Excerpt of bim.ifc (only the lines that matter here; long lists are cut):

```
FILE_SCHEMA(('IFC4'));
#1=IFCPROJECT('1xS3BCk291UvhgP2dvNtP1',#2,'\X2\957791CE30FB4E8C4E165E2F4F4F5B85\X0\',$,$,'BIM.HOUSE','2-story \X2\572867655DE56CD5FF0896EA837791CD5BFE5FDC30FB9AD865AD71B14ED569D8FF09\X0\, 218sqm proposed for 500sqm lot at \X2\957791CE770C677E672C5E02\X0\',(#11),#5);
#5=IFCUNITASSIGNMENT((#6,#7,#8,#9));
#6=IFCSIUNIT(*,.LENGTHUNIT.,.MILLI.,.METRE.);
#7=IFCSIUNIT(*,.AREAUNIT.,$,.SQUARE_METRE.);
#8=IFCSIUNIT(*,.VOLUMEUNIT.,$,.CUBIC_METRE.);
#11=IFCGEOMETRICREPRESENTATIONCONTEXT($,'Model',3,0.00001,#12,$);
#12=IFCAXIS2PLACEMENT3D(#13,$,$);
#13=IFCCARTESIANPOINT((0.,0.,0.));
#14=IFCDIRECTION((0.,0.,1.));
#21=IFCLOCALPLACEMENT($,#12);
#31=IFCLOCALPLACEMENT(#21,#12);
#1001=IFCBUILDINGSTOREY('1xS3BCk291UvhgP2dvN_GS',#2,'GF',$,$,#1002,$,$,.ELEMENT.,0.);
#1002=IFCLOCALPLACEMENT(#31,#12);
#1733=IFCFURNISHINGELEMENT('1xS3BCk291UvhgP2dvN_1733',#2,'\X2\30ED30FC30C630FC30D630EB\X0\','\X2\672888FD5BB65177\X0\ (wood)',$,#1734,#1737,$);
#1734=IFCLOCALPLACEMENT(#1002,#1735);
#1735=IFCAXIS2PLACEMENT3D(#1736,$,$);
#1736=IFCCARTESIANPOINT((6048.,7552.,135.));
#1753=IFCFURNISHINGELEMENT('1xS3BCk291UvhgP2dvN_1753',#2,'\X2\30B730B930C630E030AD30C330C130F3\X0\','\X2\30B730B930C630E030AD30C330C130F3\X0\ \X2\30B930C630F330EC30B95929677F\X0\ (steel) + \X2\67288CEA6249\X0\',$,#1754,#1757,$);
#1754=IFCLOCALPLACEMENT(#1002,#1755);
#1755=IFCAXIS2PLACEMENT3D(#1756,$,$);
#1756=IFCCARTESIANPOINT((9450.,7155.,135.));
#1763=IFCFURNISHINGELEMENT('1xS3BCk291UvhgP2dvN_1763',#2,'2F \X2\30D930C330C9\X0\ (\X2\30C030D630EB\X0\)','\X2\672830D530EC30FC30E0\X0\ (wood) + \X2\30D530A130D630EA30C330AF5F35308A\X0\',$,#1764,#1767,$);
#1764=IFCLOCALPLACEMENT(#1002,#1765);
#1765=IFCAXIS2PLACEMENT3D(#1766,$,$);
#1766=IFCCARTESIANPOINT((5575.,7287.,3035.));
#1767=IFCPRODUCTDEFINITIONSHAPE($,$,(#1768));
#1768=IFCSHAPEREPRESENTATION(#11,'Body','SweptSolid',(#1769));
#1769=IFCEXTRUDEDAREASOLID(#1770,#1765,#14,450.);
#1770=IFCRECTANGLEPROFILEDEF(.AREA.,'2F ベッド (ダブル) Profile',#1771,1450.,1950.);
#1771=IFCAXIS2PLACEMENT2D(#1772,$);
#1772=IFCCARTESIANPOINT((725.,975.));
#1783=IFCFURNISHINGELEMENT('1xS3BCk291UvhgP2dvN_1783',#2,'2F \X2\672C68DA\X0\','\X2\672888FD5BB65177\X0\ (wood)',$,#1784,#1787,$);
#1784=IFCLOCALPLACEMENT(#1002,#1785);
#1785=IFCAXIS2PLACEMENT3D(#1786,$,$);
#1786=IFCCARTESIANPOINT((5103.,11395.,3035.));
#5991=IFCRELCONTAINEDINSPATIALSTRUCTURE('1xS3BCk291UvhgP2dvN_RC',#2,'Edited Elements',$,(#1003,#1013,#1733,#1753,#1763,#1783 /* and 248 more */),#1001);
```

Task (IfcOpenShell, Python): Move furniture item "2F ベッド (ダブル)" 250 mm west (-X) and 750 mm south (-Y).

```python
import ifcopenshell
import ifcopenshell.api.geometry
import ifcopenshell.util.placement

model = ifcopenshell.open("bim.ifc")

item = model.by_guid("1xS3BCk291UvhgP2dvN_1763")
matrix = ifcopenshell.util.placement.get_local_placement(item.ObjectPlacement)
matrix[0, 3] -= 250.0
matrix[1, 3] -= 750.0
ifcopenshell.api.geometry.edit_object_placement(model, product=item, matrix=matrix, is_si=False)

print(ifcopenshell.util.placement.get_local_placement(item.ObjectPlacement).round(3) + 0.0)

model.write("bim_rev.ifc")
```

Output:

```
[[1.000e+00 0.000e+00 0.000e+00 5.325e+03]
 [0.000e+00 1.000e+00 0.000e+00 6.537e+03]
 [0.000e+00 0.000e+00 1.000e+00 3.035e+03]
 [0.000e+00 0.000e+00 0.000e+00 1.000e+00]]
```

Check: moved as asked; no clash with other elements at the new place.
